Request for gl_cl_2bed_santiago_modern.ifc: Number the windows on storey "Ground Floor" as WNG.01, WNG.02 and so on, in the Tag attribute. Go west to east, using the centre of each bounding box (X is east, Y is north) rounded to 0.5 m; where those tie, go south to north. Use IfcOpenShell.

First a look at what the model holds.

```python
import ifcopenshell
import ifcopenshell.util.element
import ifcopenshell.util.placement

model = ifcopenshell.open("gl_cl_2bed_santiago_modern.ifc")
print(model.schema)
storey = next(s for s in model.by_type("IfcBuildingStorey") if s.Name == "Ground Floor")
windows = [e for e in ifcopenshell.util.element.get_decomposition(storey) if e.is_a("IfcWindow")]
for e in sorted(windows, key=lambda e: e.id()):
    origin = ifcopenshell.util.placement.get_local_placement(e.ObjectPlacement)[:3, 3]
    print(e.id(), e.Tag, e.Name, origin.round(2) + 0.0, sep=" | ")
```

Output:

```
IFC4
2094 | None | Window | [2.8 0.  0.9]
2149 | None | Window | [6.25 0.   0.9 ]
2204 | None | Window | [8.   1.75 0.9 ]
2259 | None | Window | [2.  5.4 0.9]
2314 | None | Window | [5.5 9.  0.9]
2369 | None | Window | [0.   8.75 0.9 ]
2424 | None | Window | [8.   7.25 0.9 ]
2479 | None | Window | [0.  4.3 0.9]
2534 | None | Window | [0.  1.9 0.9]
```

```python
import ifcopenshell
import ifcopenshell.geom
import ifcopenshell.util.element
import ifcopenshell.util.shape

model = ifcopenshell.open("gl_cl_2bed_santiago_modern.ifc")
settings = ifcopenshell.geom.settings()
settings.set("use-world-coords", True)


def centre(element):
    shape = ifcopenshell.geom.create_shape(settings, element)
    return ifcopenshell.util.shape.get_bbox_centroid(shape.geometry)


storey = next(s for s in model.by_type("IfcBuildingStorey") if s.Name == "Ground Floor")
windows = [e for e in ifcopenshell.util.element.get_decomposition(storey) if e.is_a("IfcWindow")]

# Insertion points can sit at a corner or the storey origin, so sort by the geometry (in metres).
centres = {e: centre(e) for e in windows}
windows.sort(key=lambda e: (round(centres[e][0] / 0.5), centres[e][1]))

for i, e in enumerate(windows, start=1):
    number = f"WNG.{i:02d}"
    e.Tag = number
    print(e.id(), number)

model.write("gl_cl_2bed_santiago_modern_edited.ifc")
```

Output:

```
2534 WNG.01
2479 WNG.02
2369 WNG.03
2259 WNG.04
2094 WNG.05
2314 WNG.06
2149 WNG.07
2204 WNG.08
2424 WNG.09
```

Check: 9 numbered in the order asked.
